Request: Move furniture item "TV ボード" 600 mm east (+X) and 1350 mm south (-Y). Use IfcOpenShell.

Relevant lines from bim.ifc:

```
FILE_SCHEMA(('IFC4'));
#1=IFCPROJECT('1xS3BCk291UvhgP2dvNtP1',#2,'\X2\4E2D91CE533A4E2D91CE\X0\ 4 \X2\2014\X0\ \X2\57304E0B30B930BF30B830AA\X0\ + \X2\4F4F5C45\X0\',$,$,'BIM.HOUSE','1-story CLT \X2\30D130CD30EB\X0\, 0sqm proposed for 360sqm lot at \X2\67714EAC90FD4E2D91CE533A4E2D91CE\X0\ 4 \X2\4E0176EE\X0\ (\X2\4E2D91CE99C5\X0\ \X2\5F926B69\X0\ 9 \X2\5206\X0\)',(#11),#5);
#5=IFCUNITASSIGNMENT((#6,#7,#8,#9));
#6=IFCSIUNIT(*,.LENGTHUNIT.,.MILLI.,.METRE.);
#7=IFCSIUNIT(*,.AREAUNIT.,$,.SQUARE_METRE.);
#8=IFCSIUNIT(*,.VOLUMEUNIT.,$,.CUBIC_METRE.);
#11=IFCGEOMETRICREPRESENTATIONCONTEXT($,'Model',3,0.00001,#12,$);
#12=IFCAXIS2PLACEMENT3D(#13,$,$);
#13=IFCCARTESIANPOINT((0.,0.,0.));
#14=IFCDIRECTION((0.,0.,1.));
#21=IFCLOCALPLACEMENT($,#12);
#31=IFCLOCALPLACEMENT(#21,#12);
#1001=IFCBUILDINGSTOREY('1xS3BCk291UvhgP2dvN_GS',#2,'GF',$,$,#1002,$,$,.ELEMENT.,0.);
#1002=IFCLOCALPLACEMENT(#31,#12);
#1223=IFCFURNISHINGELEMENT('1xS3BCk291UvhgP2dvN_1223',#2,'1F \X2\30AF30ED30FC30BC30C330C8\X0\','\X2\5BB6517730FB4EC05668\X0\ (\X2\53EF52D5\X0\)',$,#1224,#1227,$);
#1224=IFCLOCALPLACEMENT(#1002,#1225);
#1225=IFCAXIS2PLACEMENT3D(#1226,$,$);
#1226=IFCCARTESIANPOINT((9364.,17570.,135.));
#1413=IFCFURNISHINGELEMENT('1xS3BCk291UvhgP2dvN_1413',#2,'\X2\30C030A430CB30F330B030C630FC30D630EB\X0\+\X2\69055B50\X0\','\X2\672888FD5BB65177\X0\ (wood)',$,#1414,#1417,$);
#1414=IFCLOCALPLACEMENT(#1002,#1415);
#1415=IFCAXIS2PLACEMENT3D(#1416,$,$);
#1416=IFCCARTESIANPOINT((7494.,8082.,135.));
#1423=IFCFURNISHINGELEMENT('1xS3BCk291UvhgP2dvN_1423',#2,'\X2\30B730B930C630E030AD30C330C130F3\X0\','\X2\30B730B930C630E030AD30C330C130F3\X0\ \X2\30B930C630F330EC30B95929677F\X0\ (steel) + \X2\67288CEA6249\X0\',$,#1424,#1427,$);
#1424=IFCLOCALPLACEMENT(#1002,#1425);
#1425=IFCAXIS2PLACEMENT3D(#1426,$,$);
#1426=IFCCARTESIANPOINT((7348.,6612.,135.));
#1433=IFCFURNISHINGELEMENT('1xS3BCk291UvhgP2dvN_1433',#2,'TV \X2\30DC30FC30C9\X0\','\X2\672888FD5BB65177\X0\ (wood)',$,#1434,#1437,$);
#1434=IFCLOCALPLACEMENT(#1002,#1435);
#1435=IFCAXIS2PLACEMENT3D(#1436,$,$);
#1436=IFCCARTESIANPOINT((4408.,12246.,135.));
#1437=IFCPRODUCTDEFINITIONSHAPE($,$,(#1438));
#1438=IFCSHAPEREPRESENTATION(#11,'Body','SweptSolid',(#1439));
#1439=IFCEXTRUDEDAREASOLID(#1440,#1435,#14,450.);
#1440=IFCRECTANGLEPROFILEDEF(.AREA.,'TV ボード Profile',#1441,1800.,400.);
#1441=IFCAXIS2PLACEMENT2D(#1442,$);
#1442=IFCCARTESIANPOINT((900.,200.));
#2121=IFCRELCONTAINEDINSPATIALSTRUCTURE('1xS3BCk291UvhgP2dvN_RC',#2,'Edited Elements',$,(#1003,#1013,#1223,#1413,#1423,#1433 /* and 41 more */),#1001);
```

```python
import ifcopenshell
import ifcopenshell.api.geometry
import ifcopenshell.util.placement
import ifcopenshell.util.unit

model = ifcopenshell.open("bim.ifc")
unit_scale = ifcopenshell.util.unit.calculate_unit_scale(model)

item = model.by_guid("1xS3BCk291UvhgP2dvN_1433")
matrix = ifcopenshell.util.placement.get_local_placement(item.ObjectPlacement)
matrix[0, 3] += 0.6 / unit_scale
matrix[1, 3] -= 1.35 / unit_scale
ifcopenshell.api.geometry.edit_object_placement(model, product=item, matrix=matrix, is_si=False)

print(ifcopenshell.util.placement.get_local_placement(item.ObjectPlacement).round(3) + 0.0)

model.write("bim-out.ifc")
```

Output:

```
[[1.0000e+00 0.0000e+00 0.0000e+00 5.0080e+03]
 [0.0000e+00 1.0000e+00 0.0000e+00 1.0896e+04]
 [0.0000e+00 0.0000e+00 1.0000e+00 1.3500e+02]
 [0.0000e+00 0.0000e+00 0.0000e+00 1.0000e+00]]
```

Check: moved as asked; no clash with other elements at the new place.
